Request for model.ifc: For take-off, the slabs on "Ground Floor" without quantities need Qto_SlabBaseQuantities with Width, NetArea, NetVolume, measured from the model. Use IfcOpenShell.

First a look at what the model holds.

```python
import ifcopenshell
import ifcopenshell.util.element
import ifcopenshell.util.unit

model = ifcopenshell.open("model.ifc")
print(model.schema)
for unit_type in ("LENGTHUNIT", "AREAUNIT", "VOLUMEUNIT"):
    print(unit_type, ifcopenshell.util.unit.calculate_unit_scale(model, unit_type))
storey = next(s for s in model.by_type("IfcBuildingStorey") if s.Name == "Ground Floor")
slabs = [e for e in ifcopenshell.util.element.get_decomposition(storey) if e.is_a("IfcSlab")]
for e in sorted(slabs, key=lambda e: e.id()):
    print(e.id(), e.is_a(), e.Name, list(ifcopenshell.util.element.get_psets(e, qtos_only=True)), sep=" | ")
```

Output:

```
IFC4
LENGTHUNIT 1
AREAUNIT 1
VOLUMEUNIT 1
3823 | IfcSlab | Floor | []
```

```python
import ifcopenshell
import ifcopenshell.api.pset
import ifcopenshell.geom
import ifcopenshell.util.element
import ifcopenshell.util.shape
import ifcopenshell.util.unit

model = ifcopenshell.open("model.ifc")
unit_scale = ifcopenshell.util.unit.calculate_unit_scale(model)
area_scale = ifcopenshell.util.unit.calculate_unit_scale(model, "AREAUNIT")
volume_scale = ifcopenshell.util.unit.calculate_unit_scale(model, "VOLUMEUNIT")
settings = ifcopenshell.geom.settings()

storey = next(s for s in model.by_type("IfcBuildingStorey") if s.Name == "Ground Floor")
slabs = [e for e in ifcopenshell.util.element.get_decomposition(storey) if e.is_a("IfcSlab")]

for e in sorted(slabs, key=lambda e: e.id()):
    if ifcopenshell.util.element.get_psets(e, qtos_only=True, should_inherit=False):
        continue
    # Geometry comes back in metres, in the element's own axes.
    shape = ifcopenshell.geom.create_shape(settings, e)
    values = {
        "Width": ifcopenshell.util.shape.get_z(shape.geometry) / unit_scale,
        "NetArea": ifcopenshell.util.shape.get_footprint_area(shape.geometry) / area_scale,
        "NetVolume": ifcopenshell.util.shape.get_volume(shape.geometry) / volume_scale,
    }
    qto = ifcopenshell.api.pset.add_qto(model, product=e, name="Qto_SlabBaseQuantities")
    ifcopenshell.api.pset.edit_qto(model, qto=qto, properties=values)
    print(e.id(), {k: round(v, 3) for k, v in values.items()})

model.write("model_updated.ifc")
```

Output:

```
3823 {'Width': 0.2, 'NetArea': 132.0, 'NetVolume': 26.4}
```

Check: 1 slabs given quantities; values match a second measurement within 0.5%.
